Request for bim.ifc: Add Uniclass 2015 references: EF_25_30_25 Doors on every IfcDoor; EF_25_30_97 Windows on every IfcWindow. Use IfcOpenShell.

First a look at what the model holds.

```python
import ifcopenshell

model = ifcopenshell.open("bim.ifc")
print(model.schema)
print("classifications:", [c.Name for c in model.by_type("IfcClassification")])
for ifc_class in ("IfcDoor", "IfcRoof", "IfcStair", "IfcWall", "IfcWindow"):
    print(ifc_class, len(model.by_type(ifc_class)))
```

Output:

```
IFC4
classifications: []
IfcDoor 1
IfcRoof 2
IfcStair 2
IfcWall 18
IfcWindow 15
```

```python
import ifcopenshell
import ifcopenshell.api.classification

model = ifcopenshell.open("bim.ifc")

system = ifcopenshell.api.classification.add_classification(model, classification="Uniclass 2015")

codes = {
    "IfcDoor": ("EF_25_30_25", "Doors"),
    "IfcWindow": ("EF_25_30_97", "Windows"),
}
for ifc_class, (code, name) in codes.items():
    products = model.by_type(ifc_class)
    ifcopenshell.api.classification.add_reference(
        model, products=products, classification=system, identification=code, name=name
    )
    print(code, len(products))

model.write("bim-out.ifc")
```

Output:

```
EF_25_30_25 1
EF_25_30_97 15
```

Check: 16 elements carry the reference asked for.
